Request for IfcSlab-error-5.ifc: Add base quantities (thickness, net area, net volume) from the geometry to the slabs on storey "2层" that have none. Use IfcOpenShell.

First a look at what the model holds.

```python
import ifcopenshell
import ifcopenshell.util.element
import ifcopenshell.util.unit

model = ifcopenshell.open("IfcSlab-error-5.ifc")
print(model.schema)
for unit_type in ("LENGTHUNIT", "AREAUNIT", "VOLUMEUNIT"):
    print(unit_type, ifcopenshell.util.unit.calculate_unit_scale(model, unit_type))
storey = next(s for s in model.by_type("IfcBuildingStorey") if s.Name == "2层")
slabs = [e for e in ifcopenshell.util.element.get_decomposition(storey) if e.is_a("IfcSlab")]
for e in sorted(slabs, key=lambda e: e.id()):
    print(e.id(), e.is_a(), e.Name, list(ifcopenshell.util.element.get_psets(e, qtos_only=True)), sep=" | ")
```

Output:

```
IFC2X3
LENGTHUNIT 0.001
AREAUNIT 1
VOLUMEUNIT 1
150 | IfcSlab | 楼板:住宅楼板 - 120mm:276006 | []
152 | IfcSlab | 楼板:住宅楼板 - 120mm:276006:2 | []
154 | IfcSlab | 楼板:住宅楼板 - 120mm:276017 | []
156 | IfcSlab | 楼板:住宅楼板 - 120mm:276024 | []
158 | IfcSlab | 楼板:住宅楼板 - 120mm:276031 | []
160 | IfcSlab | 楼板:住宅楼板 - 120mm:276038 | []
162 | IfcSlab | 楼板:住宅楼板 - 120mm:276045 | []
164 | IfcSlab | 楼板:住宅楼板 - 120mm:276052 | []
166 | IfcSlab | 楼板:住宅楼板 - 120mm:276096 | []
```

```python
import ifcopenshell
import ifcopenshell.api.pset
import ifcopenshell.geom
import ifcopenshell.util.element
import ifcopenshell.util.shape
import ifcopenshell.util.unit

model = ifcopenshell.open("IfcSlab-error-5.ifc")
unit_scale = ifcopenshell.util.unit.calculate_unit_scale(model)
area_scale = ifcopenshell.util.unit.calculate_unit_scale(model, "AREAUNIT")
volume_scale = ifcopenshell.util.unit.calculate_unit_scale(model, "VOLUMEUNIT")
settings = ifcopenshell.geom.settings()

storey = next(s for s in model.by_type("IfcBuildingStorey") if s.Name == "2层")
slabs = [e for e in ifcopenshell.util.element.get_decomposition(storey) if e.is_a("IfcSlab")]

for e in sorted(slabs, key=lambda e: e.id()):
    if ifcopenshell.util.element.get_psets(e, qtos_only=True, should_inherit=False):
        continue
    # Geometry comes back in metres, in the element's own axes.
    shape = ifcopenshell.geom.create_shape(settings, e)
    values = {
        "Width": ifcopenshell.util.shape.get_z(shape.geometry) / unit_scale,
        "NetArea": ifcopenshell.util.shape.get_footprint_area(shape.geometry) / area_scale,
        "NetVolume": ifcopenshell.util.shape.get_volume(shape.geometry) / volume_scale,
    }
    qto = ifcopenshell.api.pset.add_qto(model, product=e, name="BaseQuantities")
    ifcopenshell.api.pset.edit_qto(model, qto=qto, properties=values)
    print(e.id(), {k: round(v, 3) for k, v in values.items()})

model.write("IfcSlab-error-5_updated.ifc")
```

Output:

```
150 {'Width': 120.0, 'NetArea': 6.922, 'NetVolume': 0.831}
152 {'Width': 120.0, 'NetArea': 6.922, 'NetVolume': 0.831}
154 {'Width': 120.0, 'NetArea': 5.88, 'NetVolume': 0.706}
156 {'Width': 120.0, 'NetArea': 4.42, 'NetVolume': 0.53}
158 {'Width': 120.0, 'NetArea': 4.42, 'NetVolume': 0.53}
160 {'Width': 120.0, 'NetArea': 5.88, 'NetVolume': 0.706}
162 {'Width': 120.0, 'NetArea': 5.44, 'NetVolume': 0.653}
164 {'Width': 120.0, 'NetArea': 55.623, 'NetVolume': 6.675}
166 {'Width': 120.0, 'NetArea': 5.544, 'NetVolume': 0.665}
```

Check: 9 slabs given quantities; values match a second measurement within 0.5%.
